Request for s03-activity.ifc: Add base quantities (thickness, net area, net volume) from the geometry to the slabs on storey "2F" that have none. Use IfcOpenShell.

First a look at what the model holds.

```python
import ifcopenshell
import ifcopenshell.util.element
import ifcopenshell.util.unit

model = ifcopenshell.open("s03-activity.ifc")
print(model.schema)
for unit_type in ("LENGTHUNIT", "AREAUNIT", "VOLUMEUNIT"):
    print(unit_type, ifcopenshell.util.unit.calculate_unit_scale(model, unit_type))
storey = next(s for s in model.by_type("IfcBuildingStorey") if s.Name == "2F")
slabs = [e for e in ifcopenshell.util.element.get_decomposition(storey) if e.is_a("IfcSlab")]
for e in sorted(slabs, key=lambda e: e.id()):
    print(e.id(), e.is_a(), e.Name, list(ifcopenshell.util.element.get_psets(e, qtos_only=True)), sep=" | ")
```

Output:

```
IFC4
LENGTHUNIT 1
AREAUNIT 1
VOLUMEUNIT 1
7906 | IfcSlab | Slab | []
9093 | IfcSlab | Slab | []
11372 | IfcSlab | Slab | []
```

```python
import ifcopenshell
import ifcopenshell.api.pset
import ifcopenshell.geom
import ifcopenshell.util.element
import ifcopenshell.util.shape
import ifcopenshell.util.unit

model = ifcopenshell.open("s03-activity.ifc")
unit_scale = ifcopenshell.util.unit.calculate_unit_scale(model)
area_scale = ifcopenshell.util.unit.calculate_unit_scale(model, "AREAUNIT")
volume_scale = ifcopenshell.util.unit.calculate_unit_scale(model, "VOLUMEUNIT")
settings = ifcopenshell.geom.settings()

storey = next(s for s in model.by_type("IfcBuildingStorey") if s.Name == "2F")
slabs = [e for e in ifcopenshell.util.element.get_decomposition(storey) if e.is_a("IfcSlab")]

for e in sorted(slabs, key=lambda e: e.id()):
    if ifcopenshell.util.element.get_psets(e, qtos_only=True, should_inherit=False):
        continue
    # Geometry comes back in metres, in the element's own axes.
    shape = ifcopenshell.geom.create_shape(settings, e)
    values = {
        "Width": ifcopenshell.util.shape.get_z(shape.geometry) / unit_scale,
        "NetArea": ifcopenshell.util.shape.get_footprint_area(shape.geometry) / area_scale,
        "NetVolume": ifcopenshell.util.shape.get_volume(shape.geometry) / volume_scale,
    }
    qto = ifcopenshell.api.pset.add_qto(model, product=e, name="Qto_SlabBaseQuantities")
    ifcopenshell.api.pset.edit_qto(model, qto=qto, properties=values)
    print(e.id(), {k: round(v, 3) for k, v in values.items()})

model.write("s03-activity_v2.ifc")
```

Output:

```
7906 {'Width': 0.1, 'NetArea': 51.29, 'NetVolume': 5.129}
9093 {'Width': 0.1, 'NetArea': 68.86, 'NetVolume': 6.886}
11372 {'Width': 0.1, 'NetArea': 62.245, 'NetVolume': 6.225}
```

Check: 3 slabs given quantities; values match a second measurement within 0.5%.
